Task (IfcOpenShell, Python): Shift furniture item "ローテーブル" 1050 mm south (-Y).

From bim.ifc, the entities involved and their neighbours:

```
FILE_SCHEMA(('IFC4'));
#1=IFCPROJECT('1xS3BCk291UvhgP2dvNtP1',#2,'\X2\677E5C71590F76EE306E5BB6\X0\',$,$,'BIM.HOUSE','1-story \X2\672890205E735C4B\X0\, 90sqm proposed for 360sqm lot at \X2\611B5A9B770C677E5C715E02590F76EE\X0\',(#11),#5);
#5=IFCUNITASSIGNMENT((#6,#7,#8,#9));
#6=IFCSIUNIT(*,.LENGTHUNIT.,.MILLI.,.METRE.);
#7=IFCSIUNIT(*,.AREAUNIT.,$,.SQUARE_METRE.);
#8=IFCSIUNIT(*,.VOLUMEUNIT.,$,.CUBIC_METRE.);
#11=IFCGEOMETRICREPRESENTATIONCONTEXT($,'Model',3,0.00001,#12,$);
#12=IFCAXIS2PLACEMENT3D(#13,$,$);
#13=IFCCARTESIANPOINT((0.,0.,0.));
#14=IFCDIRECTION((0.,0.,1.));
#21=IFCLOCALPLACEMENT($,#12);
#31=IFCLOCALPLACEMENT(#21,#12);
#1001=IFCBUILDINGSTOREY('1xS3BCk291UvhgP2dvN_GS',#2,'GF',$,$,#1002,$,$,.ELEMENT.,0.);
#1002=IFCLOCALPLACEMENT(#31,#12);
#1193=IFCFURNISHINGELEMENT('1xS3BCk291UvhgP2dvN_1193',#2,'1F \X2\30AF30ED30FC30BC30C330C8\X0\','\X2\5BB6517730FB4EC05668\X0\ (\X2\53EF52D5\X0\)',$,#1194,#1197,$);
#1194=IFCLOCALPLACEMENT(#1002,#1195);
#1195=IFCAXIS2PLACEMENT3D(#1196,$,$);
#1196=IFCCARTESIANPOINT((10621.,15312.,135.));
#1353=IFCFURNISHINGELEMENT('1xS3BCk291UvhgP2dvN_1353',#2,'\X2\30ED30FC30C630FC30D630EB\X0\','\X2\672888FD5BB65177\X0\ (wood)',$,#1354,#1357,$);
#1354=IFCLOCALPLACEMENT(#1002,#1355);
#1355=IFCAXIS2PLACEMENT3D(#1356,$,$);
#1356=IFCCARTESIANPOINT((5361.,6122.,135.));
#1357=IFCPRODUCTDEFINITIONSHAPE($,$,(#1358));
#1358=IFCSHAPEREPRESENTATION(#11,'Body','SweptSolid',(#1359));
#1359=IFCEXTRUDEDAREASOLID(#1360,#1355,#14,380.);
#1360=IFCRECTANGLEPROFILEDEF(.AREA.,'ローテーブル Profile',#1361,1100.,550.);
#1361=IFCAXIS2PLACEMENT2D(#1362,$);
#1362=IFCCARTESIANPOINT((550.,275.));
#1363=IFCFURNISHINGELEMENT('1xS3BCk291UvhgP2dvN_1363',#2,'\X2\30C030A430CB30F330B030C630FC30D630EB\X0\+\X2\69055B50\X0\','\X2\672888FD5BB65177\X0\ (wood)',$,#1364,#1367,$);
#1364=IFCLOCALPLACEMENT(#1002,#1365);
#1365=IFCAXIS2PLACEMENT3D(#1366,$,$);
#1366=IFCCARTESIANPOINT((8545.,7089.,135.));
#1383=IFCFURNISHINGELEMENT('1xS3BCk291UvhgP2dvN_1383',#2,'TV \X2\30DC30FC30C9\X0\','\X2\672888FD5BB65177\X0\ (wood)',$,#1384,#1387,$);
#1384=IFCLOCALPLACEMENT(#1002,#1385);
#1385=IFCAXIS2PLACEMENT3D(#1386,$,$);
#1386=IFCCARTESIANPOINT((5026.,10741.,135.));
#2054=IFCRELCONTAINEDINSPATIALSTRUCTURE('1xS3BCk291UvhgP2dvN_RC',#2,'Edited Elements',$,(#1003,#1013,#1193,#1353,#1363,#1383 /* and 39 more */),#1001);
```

```python
import ifcopenshell
import ifcopenshell.api.geometry
import ifcopenshell.util.placement

model = ifcopenshell.open("bim.ifc")

item = model.by_id(1353)
matrix = ifcopenshell.util.placement.get_local_placement(item.ObjectPlacement)
matrix[1, 3] -= 1050.0
ifcopenshell.api.geometry.edit_object_placement(model, product=item, matrix=matrix, is_si=False)

print(ifcopenshell.util.placement.get_local_placement(item.ObjectPlacement).round(3) + 0.0)

model.write("bim_rev.ifc")
```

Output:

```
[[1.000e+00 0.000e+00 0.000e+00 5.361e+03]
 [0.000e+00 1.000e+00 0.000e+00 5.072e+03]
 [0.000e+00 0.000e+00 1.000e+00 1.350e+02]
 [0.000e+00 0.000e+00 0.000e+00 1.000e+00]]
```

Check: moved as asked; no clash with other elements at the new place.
